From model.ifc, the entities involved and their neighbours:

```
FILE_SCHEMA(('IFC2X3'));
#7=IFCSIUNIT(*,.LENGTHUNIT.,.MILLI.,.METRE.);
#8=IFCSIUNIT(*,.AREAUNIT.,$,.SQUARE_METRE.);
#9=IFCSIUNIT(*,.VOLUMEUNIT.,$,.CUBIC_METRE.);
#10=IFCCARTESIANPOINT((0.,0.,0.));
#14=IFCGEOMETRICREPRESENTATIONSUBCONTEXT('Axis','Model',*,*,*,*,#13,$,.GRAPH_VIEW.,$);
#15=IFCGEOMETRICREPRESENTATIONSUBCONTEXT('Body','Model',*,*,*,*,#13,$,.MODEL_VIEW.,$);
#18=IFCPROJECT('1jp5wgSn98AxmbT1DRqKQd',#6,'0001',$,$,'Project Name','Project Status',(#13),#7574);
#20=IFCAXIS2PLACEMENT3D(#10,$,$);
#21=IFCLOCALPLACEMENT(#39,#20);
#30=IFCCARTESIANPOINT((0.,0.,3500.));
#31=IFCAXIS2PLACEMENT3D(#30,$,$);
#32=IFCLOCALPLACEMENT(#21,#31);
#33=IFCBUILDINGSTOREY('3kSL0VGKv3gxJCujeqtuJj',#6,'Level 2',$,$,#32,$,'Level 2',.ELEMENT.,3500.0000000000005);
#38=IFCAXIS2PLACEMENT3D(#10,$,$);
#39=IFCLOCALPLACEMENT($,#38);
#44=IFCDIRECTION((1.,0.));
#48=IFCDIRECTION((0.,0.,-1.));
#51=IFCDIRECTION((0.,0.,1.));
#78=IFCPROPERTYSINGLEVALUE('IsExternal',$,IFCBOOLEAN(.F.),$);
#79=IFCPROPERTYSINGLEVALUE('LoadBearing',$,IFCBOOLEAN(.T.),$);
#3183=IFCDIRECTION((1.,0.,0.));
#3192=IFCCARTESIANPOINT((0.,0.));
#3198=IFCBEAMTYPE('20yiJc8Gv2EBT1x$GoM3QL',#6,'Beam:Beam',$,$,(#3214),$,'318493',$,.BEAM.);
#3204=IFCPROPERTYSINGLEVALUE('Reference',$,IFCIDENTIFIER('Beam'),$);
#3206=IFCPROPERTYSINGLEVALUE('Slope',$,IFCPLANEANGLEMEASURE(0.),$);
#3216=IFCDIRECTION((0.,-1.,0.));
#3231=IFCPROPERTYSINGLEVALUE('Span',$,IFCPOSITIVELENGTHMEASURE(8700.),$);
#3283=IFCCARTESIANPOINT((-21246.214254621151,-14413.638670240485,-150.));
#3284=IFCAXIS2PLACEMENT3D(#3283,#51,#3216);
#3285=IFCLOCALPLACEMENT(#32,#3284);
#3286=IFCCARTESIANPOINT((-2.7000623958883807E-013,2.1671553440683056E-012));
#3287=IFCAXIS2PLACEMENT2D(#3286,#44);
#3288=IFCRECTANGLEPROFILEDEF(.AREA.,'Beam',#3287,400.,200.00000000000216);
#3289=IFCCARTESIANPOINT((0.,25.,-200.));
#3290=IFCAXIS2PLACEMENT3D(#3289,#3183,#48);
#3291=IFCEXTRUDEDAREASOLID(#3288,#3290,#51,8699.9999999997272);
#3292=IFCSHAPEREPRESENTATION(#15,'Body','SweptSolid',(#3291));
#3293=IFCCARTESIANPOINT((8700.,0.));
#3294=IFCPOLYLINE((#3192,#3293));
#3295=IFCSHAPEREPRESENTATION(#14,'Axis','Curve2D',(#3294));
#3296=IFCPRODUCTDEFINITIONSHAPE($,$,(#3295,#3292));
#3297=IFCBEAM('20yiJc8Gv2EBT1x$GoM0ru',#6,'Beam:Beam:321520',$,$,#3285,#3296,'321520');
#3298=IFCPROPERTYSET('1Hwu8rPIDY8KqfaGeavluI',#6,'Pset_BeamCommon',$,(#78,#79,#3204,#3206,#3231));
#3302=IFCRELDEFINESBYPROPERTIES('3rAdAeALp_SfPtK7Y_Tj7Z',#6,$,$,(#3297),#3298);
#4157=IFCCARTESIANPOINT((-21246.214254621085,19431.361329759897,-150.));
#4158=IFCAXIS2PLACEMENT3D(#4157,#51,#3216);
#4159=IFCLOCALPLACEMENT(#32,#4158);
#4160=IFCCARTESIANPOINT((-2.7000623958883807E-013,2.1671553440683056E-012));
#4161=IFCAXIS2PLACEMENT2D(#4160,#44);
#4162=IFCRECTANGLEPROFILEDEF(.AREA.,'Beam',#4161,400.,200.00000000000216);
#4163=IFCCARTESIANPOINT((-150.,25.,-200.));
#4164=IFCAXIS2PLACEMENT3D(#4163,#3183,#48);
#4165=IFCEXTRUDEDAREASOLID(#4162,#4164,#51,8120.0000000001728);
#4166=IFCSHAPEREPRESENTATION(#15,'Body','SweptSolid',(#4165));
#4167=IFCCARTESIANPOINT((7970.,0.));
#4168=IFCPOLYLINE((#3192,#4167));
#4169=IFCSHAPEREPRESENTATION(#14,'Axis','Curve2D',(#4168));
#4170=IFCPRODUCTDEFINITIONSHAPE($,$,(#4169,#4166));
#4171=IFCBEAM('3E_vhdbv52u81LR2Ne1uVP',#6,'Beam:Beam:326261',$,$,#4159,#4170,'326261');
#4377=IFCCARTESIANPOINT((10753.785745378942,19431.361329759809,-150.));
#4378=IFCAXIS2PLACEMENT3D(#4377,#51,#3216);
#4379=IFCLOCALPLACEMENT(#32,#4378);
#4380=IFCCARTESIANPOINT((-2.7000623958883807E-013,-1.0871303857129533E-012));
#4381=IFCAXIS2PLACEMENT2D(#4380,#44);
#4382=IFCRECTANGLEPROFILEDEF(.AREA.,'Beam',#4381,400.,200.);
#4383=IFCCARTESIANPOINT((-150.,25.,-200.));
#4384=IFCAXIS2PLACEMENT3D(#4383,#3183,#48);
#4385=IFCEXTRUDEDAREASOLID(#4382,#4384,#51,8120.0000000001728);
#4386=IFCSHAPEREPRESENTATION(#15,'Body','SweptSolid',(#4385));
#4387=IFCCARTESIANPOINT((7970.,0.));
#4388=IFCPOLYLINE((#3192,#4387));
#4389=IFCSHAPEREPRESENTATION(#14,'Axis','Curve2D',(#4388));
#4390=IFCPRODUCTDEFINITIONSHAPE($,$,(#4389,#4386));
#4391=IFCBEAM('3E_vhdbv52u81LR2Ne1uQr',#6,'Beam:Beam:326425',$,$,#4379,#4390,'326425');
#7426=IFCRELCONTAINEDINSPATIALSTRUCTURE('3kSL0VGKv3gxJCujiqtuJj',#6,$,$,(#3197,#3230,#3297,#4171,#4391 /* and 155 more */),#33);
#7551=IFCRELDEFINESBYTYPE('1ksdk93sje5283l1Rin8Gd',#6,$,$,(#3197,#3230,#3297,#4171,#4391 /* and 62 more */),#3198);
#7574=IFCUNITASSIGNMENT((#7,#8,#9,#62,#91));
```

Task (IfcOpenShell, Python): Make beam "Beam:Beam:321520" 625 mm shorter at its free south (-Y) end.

```python
import numpy as np
import ifcopenshell
import ifcopenshell.api.pset
import ifcopenshell.util.element
import ifcopenshell.util.representation

model = ifcopenshell.open("model.ifc")

member = model.by_id(3297)
change = -625.0

# The extrusion runs towards the end named, so only its depth changes.
body = ifcopenshell.util.representation.get_representation(member, "Model", "Body")
solid = body.Items[0]
old_length = solid.Depth
solid.Depth += change

# Move the axis end point with it.
axis = next(r for r in member.Representation.Representations if r.RepresentationIdentifier == "Axis").Items[0]
start, end = (np.array(p.Coordinates) for p in axis.Points)
end = end + (end - start) / np.linalg.norm(end - start) * change
point = model.createIfcCartesianPoint(end.tolist())
axis.Points = [axis.Points[0], point]

# Update the stored length and volume.
pset = model.by_id(ifcopenshell.util.element.get_pset(member, "Pset_BeamCommon", should_inherit=False)["id"])
ifcopenshell.api.pset.edit_pset(model, pset=pset, properties={
    "Span": model.create_entity("IfcPositiveLengthMeasure", solid.Depth),
})

print(f"length {old_length:g} -> {solid.Depth:g}")

model.write("model_updated.ifc")
```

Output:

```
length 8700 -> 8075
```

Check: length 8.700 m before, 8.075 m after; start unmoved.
